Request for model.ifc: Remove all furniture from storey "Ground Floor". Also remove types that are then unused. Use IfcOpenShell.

First a look at what the model holds.

```python
import ifcopenshell
import ifcopenshell.util.element

model = ifcopenshell.open("model.ifc")
print(model.schema)
storey = next(s for s in model.by_type("IfcBuildingStorey") if s.Name == "Ground Floor")
furniture = [e for e in ifcopenshell.util.element.get_decomposition(storey) if e.is_a("IfcFurnishingElement")]
seen = {}
for e in furniture:
    element_type = ifcopenshell.util.element.get_type(e)
    name = element_type.Name if element_type not in (None, e) else None
    seen[name] = seen.get(name, 0) + 1
for name, count in sorted(seen.items(), key=str):
    print(count, "x", name)
```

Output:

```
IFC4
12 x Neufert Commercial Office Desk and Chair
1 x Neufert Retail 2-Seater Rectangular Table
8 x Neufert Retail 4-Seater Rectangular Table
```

```python
import ifcopenshell
import ifcopenshell.api.root
import ifcopenshell.util.element

model = ifcopenshell.open("model.ifc")

storey = next(s for s in model.by_type("IfcBuildingStorey") if s.Name == "Ground Floor")
furniture = [e for e in ifcopenshell.util.element.get_decomposition(storey) if e.is_a("IfcFurnishingElement")]
types = {ifcopenshell.util.element.get_type(e) for e in furniture} - {None, *furniture}

for e in furniture:
    ifcopenshell.api.root.remove_product(model, product=e)
print(len(furniture), "removed")

unused = [t for t in types if not ifcopenshell.util.element.get_types(t)]
for t in unused:
    ifcopenshell.api.root.remove_product(model, product=t)
print(len(unused), "unused types removed")

model.write("model_rev.ifc")
```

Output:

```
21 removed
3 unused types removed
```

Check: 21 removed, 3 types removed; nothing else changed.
